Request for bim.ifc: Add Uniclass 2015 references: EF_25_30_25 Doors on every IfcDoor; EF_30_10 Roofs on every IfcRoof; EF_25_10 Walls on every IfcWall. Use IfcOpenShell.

First a look at what the model holds.

```python
import ifcopenshell

model = ifcopenshell.open("bim.ifc")
print(model.schema)
print("classifications:", [c.Name for c in model.by_type("IfcClassification")])
for ifc_class in ("IfcDoor", "IfcRoof", "IfcStair", "IfcWall", "IfcWindow"):
    print(ifc_class, len(model.by_type(ifc_class)))
```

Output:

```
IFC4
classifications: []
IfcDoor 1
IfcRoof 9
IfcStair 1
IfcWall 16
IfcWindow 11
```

```python
import ifcopenshell
import ifcopenshell.api.classification

model = ifcopenshell.open("bim.ifc")

system = ifcopenshell.api.classification.add_classification(model, classification="Uniclass 2015")

codes = {
    "IfcDoor": ("EF_25_30_25", "Doors"),
    "IfcRoof": ("EF_30_10", "Roofs"),
    "IfcWall": ("EF_25_10", "Walls"),
}
for ifc_class, (code, name) in codes.items():
    products = model.by_type(ifc_class)
    ifcopenshell.api.classification.add_reference(
        model, products=products, classification=system, identification=code, name=name
    )
    print(code, len(products))

model.write("bim_rev.ifc")
```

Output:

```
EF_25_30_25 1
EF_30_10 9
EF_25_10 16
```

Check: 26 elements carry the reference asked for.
